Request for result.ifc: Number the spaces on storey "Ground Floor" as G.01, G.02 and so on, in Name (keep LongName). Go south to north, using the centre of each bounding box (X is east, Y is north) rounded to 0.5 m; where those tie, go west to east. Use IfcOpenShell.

First a look at what the model holds.

```python
import ifcopenshell
import ifcopenshell.util.element
import ifcopenshell.util.placement

model = ifcopenshell.open("result.ifc")
print(model.schema)
storey = next(s for s in model.by_type("IfcBuildingStorey") if s.Name == "Ground Floor")
spaces = [e for e in ifcopenshell.util.element.get_decomposition(storey) if e.is_a("IfcSpace")]
for e in sorted(spaces, key=lambda e: e.id()):
    origin = ifcopenshell.util.placement.get_local_placement(e.ObjectPlacement)[:3, 3]
    print(e.id(), e.Name, e.LongName, origin.round(2) + 0.0, sep=" | ")
```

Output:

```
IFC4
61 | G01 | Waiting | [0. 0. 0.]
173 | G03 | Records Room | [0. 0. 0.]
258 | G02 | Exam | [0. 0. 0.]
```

```python
import ifcopenshell
import ifcopenshell.geom
import ifcopenshell.util.element
import ifcopenshell.util.shape

model = ifcopenshell.open("result.ifc")
settings = ifcopenshell.geom.settings()
settings.set("use-world-coords", True)


def centre(element):
    shape = ifcopenshell.geom.create_shape(settings, element)
    return ifcopenshell.util.shape.get_bbox_centroid(shape.geometry)


storey = next(s for s in model.by_type("IfcBuildingStorey") if s.Name == "Ground Floor")
spaces = [e for e in ifcopenshell.util.element.get_decomposition(storey) if e.is_a("IfcSpace")]

# Insertion points can sit at a corner or the storey origin, so sort by the geometry (in metres).
centres = {e: centre(e) for e in spaces}
spaces.sort(key=lambda e: (round(centres[e][1] / 0.5), centres[e][0]))

for i, e in enumerate(spaces, start=1):
    number = f"G.{i:02d}"
    e.Name = number
    print(e.id(), number)

model.write("result_edited.ifc")
```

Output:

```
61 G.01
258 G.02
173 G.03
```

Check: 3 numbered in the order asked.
